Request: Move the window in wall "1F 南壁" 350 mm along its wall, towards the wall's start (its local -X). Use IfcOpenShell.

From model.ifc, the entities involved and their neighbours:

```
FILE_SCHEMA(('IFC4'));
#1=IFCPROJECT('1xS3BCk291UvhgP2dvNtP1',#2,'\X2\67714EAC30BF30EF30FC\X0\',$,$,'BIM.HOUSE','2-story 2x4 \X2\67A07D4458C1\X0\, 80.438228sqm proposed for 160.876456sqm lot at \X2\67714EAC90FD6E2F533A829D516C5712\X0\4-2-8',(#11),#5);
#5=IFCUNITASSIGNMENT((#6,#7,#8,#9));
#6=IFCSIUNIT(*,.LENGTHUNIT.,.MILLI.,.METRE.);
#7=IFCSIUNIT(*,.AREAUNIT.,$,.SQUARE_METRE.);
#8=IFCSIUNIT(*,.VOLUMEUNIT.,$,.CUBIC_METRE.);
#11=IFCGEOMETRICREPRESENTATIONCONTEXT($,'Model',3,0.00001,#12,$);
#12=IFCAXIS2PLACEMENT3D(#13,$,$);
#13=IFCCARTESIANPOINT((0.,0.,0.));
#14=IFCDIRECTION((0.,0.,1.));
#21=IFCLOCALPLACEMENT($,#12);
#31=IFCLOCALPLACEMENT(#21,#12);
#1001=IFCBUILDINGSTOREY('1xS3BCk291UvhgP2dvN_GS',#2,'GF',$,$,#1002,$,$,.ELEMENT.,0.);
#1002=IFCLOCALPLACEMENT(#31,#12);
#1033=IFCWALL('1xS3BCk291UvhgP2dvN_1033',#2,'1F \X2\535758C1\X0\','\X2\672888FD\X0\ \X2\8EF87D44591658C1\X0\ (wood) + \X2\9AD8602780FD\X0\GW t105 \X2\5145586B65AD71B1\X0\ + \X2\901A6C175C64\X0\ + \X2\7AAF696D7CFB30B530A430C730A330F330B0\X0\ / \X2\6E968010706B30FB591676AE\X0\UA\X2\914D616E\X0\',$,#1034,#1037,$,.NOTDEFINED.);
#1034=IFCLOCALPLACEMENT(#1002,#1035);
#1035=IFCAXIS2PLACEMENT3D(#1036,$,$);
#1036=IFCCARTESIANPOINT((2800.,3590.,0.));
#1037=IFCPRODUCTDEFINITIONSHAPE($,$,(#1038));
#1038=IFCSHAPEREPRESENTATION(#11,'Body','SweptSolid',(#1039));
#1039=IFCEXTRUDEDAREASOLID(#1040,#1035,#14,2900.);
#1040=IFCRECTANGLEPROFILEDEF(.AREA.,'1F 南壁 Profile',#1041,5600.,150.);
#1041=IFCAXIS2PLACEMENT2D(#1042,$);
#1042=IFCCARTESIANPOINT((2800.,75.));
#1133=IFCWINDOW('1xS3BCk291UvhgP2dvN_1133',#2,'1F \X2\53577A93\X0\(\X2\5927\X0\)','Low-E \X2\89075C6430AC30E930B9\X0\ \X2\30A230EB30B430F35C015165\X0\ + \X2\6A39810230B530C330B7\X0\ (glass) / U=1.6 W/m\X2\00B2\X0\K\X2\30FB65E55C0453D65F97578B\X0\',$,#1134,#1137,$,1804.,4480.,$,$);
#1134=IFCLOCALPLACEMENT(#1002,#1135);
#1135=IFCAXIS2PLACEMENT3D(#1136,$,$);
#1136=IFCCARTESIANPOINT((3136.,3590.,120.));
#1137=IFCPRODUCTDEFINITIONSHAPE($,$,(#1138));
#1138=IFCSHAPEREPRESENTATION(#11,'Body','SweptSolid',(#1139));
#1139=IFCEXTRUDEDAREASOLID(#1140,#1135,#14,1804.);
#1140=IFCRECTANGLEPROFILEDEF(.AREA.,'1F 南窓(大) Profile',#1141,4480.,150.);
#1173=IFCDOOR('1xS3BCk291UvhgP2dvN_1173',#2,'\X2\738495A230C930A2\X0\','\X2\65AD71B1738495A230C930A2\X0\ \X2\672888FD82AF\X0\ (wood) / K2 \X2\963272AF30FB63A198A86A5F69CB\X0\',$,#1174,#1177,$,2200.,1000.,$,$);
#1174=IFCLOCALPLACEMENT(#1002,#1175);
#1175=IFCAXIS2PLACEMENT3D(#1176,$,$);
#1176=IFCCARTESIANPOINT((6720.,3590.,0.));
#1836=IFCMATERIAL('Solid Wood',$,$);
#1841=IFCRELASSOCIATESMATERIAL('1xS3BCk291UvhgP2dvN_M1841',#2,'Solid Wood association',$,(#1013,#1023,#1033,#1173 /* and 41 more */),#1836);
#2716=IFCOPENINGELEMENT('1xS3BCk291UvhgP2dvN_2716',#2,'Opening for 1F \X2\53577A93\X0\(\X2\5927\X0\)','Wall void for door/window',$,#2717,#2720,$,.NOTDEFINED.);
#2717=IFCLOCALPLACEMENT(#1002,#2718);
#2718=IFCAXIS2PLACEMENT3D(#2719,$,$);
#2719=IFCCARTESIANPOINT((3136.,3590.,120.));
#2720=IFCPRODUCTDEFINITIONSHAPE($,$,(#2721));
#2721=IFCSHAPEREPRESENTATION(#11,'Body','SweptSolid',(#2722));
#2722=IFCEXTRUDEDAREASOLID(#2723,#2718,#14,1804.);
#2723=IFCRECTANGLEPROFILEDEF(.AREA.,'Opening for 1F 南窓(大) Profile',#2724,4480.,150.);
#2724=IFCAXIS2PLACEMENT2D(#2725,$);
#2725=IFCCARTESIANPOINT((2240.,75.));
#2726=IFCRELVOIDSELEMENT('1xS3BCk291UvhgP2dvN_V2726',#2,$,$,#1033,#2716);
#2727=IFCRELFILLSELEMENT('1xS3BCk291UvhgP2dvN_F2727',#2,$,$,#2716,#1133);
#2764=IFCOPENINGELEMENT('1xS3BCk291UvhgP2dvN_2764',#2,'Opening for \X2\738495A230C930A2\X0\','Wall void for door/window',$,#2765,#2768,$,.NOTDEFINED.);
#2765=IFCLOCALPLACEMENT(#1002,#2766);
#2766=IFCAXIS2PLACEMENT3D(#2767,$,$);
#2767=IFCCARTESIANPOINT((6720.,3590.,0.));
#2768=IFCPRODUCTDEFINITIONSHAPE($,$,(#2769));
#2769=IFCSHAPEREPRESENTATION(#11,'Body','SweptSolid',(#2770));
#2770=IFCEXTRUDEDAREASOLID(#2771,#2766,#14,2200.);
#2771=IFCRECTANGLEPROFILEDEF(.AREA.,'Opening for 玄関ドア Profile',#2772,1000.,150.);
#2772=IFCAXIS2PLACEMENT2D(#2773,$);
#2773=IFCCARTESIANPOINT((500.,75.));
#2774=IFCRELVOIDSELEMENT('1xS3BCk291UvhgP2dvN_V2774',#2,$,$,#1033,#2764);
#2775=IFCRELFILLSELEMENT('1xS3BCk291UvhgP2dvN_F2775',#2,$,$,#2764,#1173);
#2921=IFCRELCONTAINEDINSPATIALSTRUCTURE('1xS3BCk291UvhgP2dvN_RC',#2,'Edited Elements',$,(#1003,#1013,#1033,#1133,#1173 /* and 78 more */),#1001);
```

```python
import ifcopenshell
import ifcopenshell.api.geometry
import ifcopenshell.util.placement

model = ifcopenshell.open("model.ifc")

window = model.by_guid("1xS3BCk291UvhgP2dvN_1133")
opening = window.FillsVoids[0].RelatingOpeningElement
wall = opening.VoidsElements[0].RelatingBuildingElement

wall_matrix = ifcopenshell.util.placement.get_local_placement(wall.ObjectPlacement)
shift = wall_matrix[:3, 0] * -350.0
before = ifcopenshell.util.placement.get_local_placement(window.ObjectPlacement)[:3, 3].copy()

# The window is not placed relative to its opening, so move both.
for product in (opening, window):
    matrix = ifcopenshell.util.placement.get_local_placement(product.ObjectPlacement)
    matrix[:3, 3] += shift
    ifcopenshell.api.geometry.edit_object_placement(model, product=product, matrix=matrix, is_si=False)

after = ifcopenshell.util.placement.get_local_placement(window.ObjectPlacement)[:3, 3]
print("window moved by", (after - before).round(3) + 0.0)

model.write("model_updated.ifc")
```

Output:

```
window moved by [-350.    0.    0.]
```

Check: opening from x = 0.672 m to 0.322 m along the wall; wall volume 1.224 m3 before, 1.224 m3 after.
